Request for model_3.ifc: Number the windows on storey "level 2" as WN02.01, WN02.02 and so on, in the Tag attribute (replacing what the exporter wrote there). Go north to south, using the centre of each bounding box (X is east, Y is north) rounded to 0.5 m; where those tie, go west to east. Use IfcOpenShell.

First a look at what the model holds.

```python
import ifcopenshell
import ifcopenshell.util.element
import ifcopenshell.util.placement

model = ifcopenshell.open("model_3.ifc")
print(model.schema)
storey = next(s for s in model.by_type("IfcBuildingStorey") if s.Name == "level 2")
windows = [e for e in ifcopenshell.util.element.get_decomposition(storey) if e.is_a("IfcWindow")]
for e in sorted(windows, key=lambda e: e.id()):
    origin = ifcopenshell.util.placement.get_local_placement(e.ObjectPlacement)[:3, 3]
    print(e.id(), e.Tag, e.Name, origin.round(2) + 0.0, sep=" | ")
```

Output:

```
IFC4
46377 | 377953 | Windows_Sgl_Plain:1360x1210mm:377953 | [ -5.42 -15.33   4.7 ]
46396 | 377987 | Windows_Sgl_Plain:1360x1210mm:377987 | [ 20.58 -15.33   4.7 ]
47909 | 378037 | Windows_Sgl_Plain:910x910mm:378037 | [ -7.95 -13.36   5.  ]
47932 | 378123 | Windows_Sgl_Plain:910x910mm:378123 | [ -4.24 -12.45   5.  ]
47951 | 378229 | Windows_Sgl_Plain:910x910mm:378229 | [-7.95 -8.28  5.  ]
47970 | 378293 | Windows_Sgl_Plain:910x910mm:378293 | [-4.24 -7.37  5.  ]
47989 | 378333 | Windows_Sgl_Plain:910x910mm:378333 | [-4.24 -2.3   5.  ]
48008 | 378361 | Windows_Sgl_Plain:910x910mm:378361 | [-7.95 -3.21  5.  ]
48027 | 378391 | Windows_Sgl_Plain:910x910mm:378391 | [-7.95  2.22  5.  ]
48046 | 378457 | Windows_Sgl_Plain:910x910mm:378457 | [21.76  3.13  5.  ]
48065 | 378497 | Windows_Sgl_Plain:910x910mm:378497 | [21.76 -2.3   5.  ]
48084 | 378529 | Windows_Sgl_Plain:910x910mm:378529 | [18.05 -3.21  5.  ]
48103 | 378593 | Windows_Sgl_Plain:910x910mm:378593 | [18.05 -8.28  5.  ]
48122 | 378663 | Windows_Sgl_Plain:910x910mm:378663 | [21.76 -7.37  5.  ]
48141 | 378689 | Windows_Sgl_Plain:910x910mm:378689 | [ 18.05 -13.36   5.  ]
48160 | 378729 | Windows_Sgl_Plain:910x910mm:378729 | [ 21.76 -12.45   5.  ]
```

```python
import ifcopenshell
import ifcopenshell.geom
import ifcopenshell.util.element
import ifcopenshell.util.shape

model = ifcopenshell.open("model_3.ifc")
settings = ifcopenshell.geom.settings()
settings.set("use-world-coords", True)


def centre(element):
    shape = ifcopenshell.geom.create_shape(settings, element)
    return ifcopenshell.util.shape.get_bbox_centroid(shape.geometry)


storey = next(s for s in model.by_type("IfcBuildingStorey") if s.Name == "level 2")
windows = [e for e in ifcopenshell.util.element.get_decomposition(storey) if e.is_a("IfcWindow")]

# Insertion points can sit at a corner or the storey origin, so sort by the geometry (in metres).
centres = {e: centre(e) for e in windows}
windows.sort(key=lambda e: (-round(centres[e][1] / 0.5), centres[e][0]))

for i, e in enumerate(windows, start=1):
    number = f"WN02.{i:02d}"
    e.Tag = number
    print(e.id(), number)

model.write("model_3_rev.ifc")
```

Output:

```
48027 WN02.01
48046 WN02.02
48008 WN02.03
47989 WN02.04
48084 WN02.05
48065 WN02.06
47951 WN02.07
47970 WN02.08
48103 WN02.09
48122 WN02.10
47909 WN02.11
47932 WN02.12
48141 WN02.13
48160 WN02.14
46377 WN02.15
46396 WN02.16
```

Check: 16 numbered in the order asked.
